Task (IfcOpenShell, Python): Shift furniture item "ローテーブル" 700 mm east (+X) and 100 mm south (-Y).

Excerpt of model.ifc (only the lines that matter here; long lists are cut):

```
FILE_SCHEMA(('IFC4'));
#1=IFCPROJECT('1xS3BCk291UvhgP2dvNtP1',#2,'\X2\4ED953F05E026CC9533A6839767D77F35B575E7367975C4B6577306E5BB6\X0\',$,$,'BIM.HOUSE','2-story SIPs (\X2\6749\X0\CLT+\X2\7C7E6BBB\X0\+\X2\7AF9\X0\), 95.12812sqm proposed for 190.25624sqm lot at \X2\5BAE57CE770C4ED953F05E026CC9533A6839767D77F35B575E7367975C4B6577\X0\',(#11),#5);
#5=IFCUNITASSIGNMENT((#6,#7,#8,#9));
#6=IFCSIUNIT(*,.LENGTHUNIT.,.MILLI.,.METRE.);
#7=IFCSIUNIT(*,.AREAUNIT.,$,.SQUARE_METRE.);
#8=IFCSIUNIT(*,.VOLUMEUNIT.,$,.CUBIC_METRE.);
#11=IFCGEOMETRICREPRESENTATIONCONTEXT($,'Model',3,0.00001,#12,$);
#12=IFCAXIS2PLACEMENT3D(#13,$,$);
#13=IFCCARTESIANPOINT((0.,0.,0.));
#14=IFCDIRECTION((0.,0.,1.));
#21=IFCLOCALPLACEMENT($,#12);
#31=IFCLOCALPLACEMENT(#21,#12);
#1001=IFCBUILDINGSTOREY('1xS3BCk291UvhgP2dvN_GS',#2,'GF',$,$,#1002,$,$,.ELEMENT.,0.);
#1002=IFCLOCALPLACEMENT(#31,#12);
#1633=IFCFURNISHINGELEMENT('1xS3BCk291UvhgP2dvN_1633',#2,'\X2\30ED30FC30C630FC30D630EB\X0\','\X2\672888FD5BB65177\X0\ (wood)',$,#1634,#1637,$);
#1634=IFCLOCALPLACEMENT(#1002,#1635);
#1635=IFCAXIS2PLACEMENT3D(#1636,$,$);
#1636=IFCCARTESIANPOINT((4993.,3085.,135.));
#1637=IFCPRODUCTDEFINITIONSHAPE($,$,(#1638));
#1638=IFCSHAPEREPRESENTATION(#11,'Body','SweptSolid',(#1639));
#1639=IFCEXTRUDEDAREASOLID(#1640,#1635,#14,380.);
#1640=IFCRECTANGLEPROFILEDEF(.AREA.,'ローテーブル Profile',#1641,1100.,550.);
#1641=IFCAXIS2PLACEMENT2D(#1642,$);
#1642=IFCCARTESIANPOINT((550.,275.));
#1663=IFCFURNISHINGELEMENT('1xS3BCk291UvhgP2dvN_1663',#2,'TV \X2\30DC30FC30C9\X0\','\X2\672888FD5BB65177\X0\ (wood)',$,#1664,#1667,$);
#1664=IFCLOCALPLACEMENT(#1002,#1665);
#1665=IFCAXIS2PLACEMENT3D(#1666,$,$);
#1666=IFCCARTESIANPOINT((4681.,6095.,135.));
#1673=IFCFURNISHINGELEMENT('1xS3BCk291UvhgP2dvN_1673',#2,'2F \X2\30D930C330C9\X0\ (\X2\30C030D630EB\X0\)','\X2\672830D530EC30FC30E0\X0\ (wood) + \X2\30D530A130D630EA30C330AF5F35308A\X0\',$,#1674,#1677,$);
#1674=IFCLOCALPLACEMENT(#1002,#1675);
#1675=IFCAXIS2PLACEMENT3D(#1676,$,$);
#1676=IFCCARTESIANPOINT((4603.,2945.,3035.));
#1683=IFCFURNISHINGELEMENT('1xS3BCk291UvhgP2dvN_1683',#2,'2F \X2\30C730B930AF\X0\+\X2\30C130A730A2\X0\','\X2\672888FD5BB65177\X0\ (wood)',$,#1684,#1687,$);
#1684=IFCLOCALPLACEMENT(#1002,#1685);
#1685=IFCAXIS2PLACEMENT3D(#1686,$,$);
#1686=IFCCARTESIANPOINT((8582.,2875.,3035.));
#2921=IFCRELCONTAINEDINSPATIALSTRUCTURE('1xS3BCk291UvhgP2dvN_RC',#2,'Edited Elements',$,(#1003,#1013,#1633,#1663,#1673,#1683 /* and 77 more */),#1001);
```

```python
import ifcopenshell
import ifcopenshell.api.geometry
import ifcopenshell.util.placement

model = ifcopenshell.open("model.ifc")

item = model.by_guid("1xS3BCk291UvhgP2dvN_1633")
matrix = ifcopenshell.util.placement.get_local_placement(item.ObjectPlacement)
matrix[0, 3] += 700.0
matrix[1, 3] -= 100.0
ifcopenshell.api.geometry.edit_object_placement(model, product=item, matrix=matrix, is_si=False)

print(ifcopenshell.util.placement.get_local_placement(item.ObjectPlacement).round(3) + 0.0)

model.write("model_updated.ifc")
```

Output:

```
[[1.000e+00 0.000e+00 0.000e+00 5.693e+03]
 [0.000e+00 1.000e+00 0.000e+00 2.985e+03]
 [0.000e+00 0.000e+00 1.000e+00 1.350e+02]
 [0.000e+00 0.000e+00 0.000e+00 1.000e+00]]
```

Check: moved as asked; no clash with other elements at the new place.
